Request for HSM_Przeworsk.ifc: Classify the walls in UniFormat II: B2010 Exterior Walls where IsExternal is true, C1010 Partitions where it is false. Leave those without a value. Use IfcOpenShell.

First a look at what the model holds.

```python
import ifcopenshell
import ifcopenshell.util.element

model = ifcopenshell.open("HSM_Przeworsk.ifc")
print(model.schema)
print("classifications:", [c.Name for c in model.by_type("IfcClassification")])
values = [ifcopenshell.util.element.get_pset(e, "Pset_WallCommon", "IsExternal") for e in model.by_type("IfcWall")]
for value in (True, False, None):
    print("IsExternal", value, values.count(value))
```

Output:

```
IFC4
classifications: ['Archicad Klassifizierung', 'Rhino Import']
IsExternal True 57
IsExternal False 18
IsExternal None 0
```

```python
import ifcopenshell
import ifcopenshell.api.classification
import ifcopenshell.util.element

model = ifcopenshell.open("HSM_Przeworsk.ifc")

system = ifcopenshell.api.classification.add_classification(model, classification="UniFormat II")

walls = model.by_type("IfcWall")
external = {e: ifcopenshell.util.element.get_pset(e, "Pset_WallCommon", "IsExternal") for e in walls}
for flag, code, name in ((True, "B2010", "Exterior Walls"), (False, "C1010", "Partitions")):
    products = [e for e in walls if external[e] is flag]
    ifcopenshell.api.classification.add_reference(
        model, products=products, classification=system, identification=code, name=name
    )
    print(code, len(products))

model.write("HSM_Przeworsk_rev.ifc")
```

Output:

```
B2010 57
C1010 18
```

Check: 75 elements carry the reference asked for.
